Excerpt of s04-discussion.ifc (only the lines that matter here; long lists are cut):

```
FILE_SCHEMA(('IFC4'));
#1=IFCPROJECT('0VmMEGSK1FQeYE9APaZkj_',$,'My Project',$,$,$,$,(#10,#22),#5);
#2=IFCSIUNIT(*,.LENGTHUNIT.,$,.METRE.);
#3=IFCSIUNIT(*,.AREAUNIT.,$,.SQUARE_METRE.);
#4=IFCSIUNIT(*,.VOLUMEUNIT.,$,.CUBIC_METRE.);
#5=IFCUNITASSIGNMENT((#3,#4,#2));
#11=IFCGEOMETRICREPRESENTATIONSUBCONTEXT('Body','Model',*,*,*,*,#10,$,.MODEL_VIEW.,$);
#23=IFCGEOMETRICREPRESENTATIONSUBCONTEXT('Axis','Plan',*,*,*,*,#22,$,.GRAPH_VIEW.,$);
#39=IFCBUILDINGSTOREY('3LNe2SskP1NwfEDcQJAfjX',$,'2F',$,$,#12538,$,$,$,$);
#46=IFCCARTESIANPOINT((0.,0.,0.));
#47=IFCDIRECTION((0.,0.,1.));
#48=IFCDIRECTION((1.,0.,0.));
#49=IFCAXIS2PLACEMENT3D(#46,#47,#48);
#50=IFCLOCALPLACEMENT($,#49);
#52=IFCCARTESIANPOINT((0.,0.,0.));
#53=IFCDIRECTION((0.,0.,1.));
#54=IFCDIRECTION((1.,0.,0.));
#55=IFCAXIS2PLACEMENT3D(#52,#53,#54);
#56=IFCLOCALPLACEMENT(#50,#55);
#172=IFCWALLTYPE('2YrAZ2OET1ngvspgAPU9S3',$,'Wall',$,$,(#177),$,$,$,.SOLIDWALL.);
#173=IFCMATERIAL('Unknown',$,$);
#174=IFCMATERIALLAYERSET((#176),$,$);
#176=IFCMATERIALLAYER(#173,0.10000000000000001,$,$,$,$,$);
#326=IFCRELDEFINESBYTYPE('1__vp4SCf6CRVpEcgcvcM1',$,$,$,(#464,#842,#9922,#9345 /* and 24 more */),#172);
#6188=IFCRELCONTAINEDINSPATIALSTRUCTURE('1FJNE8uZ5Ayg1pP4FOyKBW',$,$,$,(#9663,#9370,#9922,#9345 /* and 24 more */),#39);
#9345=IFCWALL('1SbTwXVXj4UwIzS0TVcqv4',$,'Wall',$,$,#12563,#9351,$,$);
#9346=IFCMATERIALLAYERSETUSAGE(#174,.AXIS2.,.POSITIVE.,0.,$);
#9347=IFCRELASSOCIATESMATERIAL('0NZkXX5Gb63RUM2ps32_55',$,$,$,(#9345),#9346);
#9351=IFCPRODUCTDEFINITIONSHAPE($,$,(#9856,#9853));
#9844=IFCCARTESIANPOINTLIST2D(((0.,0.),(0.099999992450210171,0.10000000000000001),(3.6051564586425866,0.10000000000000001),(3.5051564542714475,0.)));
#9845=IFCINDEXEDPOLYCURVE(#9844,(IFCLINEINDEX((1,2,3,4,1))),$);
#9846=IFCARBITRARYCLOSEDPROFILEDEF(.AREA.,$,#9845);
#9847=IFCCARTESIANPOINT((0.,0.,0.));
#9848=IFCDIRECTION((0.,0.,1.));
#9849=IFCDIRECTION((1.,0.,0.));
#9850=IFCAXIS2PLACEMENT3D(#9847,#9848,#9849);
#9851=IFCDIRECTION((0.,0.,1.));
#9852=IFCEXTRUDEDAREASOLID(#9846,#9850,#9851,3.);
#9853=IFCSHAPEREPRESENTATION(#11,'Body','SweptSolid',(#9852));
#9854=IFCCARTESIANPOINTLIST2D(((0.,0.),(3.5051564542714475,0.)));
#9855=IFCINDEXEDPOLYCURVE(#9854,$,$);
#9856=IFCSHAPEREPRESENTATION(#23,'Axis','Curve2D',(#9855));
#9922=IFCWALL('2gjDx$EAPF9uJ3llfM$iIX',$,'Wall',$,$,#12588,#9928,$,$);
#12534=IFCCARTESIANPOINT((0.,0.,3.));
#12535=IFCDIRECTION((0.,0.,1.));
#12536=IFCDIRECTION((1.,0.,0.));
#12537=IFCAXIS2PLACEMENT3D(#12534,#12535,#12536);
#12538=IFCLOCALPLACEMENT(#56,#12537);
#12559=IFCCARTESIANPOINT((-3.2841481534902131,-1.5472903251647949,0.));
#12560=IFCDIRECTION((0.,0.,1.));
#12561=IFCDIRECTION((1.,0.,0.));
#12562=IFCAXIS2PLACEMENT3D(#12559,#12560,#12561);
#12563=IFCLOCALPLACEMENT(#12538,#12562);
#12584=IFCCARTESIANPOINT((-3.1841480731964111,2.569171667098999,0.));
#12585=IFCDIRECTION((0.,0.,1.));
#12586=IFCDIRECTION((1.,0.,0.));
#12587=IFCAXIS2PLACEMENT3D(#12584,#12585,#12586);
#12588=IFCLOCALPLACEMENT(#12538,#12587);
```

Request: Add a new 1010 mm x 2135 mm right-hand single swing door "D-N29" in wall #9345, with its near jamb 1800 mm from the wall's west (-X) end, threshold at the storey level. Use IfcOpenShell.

```python
import numpy as np
import ifcopenshell
import ifcopenshell.api.feature
import ifcopenshell.api.geometry
import ifcopenshell.api.root
import ifcopenshell.api.spatial
import ifcopenshell.geom
import ifcopenshell.util.element
import ifcopenshell.util.placement
import ifcopenshell.util.representation
import ifcopenshell.util.shape
import ifcopenshell.util.unit

model = ifcopenshell.open("s04-discussion.ifc")
unit_scale = ifcopenshell.util.unit.calculate_unit_scale(model)
settings = ifcopenshell.geom.settings()


def volume(element):
    """Net volume in cubic metres, openings subtracted."""
    shape = ifcopenshell.geom.create_shape(settings, element)
    return ifcopenshell.util.shape.get_volume(shape.geometry)


wall = model.by_guid("1SbTwXVXj4UwIzS0TVcqv4")
storey = ifcopenshell.util.element.get_container(wall, ifc_class="IfcBuildingStorey")
context = ifcopenshell.util.representation.get_context(model, "Model", "Body", "MODEL_VIEW")
before = volume(wall)

width, height, from_end, sill = 1.01, 2.135, 1.8, 0.0  # metres

# The wall runs along its own X axis, and the end named is its -X end.
wall_shape = ifcopenshell.geom.create_shape(settings, wall)
x, y, z = ifcopenshell.util.shape.get_vertices(wall_shape.geometry).T
start = x.min() + from_end
face, thickness = float(y.min()), float(y.max() - y.min())
wall_matrix = ifcopenshell.util.placement.get_local_placement(wall.ObjectPlacement)
level = ifcopenshell.util.placement.get_local_placement(storey.ObjectPlacement)[2, 3]


def in_wall(x, y):
    """Placement at x, y metres in the wall's axes, at sill height."""
    matrix = wall_matrix.copy()
    matrix[:, 3] = wall_matrix @ np.array([x / unit_scale, y / unit_scale, 0.0, 1.0])
    matrix[2, 3] = level + sill / unit_scale
    return matrix


# Opening: a box that overshoots both wall faces by 50 mm.
opening = ifcopenshell.api.root.create_entity(model, ifc_class="IfcOpeningElement", predefined_type="OPENING")
box = ifcopenshell.api.geometry.add_wall_representation(
    model, context=context, length=width, height=height, thickness=thickness + 0.1
)
ifcopenshell.api.geometry.assign_representation(model, product=opening, representation=box)
ifcopenshell.api.geometry.edit_object_placement(model, product=opening, matrix=in_wall(start, face - 0.05), is_si=False)
ifcopenshell.api.feature.add_feature(model, feature=opening, element=wall)

door = ifcopenshell.api.root.create_entity(model, ifc_class="IfcDoor", name="D-N29", predefined_type="DOOR")
door.OverallWidth, door.OverallHeight = width / unit_scale, height / unit_scale
door.OperationType = "SINGLE_SWING_RIGHT"
body = ifcopenshell.api.geometry.add_door_representation(
    model,
    context=context,
    overall_width=door.OverallWidth,
    overall_height=door.OverallHeight,
    operation_type="SINGLE_SWING_RIGHT",
    lining_properties={"LiningDepth": thickness / unit_scale, "ThresholdDepth": thickness / unit_scale},
)
ifcopenshell.api.geometry.assign_representation(model, product=door, representation=body)
ifcopenshell.api.spatial.assign_container(model, products=[door], relating_structure=storey)
ifcopenshell.api.feature.add_filling(model, opening=opening, element=door)

# The lining spans the wall, so the door starts at the wall face.
ifcopenshell.api.geometry.edit_object_placement(model, product=door, matrix=in_wall(start, face), is_si=False)

after = volume(wall)

print(f"wall volume {before:.3f} -> {after:.3f} m3")

model.write("s04-discussion-out.ifc")
```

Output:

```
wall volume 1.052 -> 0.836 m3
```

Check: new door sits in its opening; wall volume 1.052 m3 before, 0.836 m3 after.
